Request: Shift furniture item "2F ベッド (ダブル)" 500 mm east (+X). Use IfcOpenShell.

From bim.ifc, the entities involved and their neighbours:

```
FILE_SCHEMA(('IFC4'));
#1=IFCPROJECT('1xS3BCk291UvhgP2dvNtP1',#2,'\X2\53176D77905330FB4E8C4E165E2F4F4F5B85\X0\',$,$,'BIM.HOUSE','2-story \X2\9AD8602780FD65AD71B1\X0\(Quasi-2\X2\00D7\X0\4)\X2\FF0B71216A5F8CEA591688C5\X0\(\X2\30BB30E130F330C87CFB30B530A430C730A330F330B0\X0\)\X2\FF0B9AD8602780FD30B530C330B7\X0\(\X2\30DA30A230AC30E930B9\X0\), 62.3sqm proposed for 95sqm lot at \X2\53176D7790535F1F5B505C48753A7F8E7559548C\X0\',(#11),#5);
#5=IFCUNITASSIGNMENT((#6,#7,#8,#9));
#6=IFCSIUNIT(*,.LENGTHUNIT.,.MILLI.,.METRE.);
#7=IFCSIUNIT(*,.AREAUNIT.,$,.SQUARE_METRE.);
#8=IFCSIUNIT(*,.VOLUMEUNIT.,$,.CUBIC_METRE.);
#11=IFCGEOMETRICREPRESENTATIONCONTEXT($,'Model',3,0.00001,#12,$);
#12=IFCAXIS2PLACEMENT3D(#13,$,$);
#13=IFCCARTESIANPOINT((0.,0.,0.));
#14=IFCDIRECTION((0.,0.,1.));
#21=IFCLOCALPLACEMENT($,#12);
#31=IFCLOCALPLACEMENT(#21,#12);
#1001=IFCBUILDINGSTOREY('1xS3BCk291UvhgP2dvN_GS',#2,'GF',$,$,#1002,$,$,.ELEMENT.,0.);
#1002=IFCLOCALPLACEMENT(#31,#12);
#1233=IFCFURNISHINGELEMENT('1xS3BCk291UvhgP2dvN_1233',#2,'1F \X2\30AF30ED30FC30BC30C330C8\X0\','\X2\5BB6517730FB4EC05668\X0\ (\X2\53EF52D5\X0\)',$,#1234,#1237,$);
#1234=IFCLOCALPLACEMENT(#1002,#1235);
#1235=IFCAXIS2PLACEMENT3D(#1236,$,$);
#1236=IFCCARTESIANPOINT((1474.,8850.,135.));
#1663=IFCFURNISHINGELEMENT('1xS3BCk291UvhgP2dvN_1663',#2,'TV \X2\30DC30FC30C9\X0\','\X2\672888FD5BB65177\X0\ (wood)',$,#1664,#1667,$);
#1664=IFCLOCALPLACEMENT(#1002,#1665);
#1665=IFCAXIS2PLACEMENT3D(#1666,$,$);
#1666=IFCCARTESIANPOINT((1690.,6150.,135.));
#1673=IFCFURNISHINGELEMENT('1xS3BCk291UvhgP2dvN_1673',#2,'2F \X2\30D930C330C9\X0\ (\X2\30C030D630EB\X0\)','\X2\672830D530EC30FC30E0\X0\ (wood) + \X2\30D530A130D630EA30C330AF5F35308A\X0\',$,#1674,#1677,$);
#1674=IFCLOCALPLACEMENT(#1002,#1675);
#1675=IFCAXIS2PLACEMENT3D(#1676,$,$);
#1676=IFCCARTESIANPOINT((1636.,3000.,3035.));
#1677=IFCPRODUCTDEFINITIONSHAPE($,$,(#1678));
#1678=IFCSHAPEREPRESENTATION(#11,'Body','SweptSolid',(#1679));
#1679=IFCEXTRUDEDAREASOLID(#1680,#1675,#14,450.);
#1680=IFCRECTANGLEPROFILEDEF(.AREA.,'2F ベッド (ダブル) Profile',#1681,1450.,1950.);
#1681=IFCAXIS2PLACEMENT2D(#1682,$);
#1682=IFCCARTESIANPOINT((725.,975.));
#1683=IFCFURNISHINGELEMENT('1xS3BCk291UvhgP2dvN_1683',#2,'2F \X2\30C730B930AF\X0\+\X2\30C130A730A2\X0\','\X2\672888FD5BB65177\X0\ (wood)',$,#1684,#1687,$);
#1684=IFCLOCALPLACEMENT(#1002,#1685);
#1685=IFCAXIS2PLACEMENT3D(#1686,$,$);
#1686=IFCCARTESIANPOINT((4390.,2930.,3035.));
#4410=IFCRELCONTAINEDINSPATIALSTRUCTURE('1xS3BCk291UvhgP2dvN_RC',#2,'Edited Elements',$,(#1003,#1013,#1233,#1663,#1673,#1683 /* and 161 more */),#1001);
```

```python
import ifcopenshell
import ifcopenshell.api.geometry
import ifcopenshell.util.placement

model = ifcopenshell.open("bim.ifc")

item = model.by_guid("1xS3BCk291UvhgP2dvN_1673")
matrix = ifcopenshell.util.placement.get_local_placement(item.ObjectPlacement)
matrix[0, 3] += 500.0
ifcopenshell.api.geometry.edit_object_placement(model, product=item, matrix=matrix, is_si=False)

print(ifcopenshell.util.placement.get_local_placement(item.ObjectPlacement).round(3) + 0.0)

model.write("bim_updated.ifc")
```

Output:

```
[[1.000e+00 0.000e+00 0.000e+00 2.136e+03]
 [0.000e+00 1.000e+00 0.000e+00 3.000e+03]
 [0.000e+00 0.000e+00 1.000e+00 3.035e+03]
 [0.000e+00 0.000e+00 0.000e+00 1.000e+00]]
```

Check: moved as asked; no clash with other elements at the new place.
